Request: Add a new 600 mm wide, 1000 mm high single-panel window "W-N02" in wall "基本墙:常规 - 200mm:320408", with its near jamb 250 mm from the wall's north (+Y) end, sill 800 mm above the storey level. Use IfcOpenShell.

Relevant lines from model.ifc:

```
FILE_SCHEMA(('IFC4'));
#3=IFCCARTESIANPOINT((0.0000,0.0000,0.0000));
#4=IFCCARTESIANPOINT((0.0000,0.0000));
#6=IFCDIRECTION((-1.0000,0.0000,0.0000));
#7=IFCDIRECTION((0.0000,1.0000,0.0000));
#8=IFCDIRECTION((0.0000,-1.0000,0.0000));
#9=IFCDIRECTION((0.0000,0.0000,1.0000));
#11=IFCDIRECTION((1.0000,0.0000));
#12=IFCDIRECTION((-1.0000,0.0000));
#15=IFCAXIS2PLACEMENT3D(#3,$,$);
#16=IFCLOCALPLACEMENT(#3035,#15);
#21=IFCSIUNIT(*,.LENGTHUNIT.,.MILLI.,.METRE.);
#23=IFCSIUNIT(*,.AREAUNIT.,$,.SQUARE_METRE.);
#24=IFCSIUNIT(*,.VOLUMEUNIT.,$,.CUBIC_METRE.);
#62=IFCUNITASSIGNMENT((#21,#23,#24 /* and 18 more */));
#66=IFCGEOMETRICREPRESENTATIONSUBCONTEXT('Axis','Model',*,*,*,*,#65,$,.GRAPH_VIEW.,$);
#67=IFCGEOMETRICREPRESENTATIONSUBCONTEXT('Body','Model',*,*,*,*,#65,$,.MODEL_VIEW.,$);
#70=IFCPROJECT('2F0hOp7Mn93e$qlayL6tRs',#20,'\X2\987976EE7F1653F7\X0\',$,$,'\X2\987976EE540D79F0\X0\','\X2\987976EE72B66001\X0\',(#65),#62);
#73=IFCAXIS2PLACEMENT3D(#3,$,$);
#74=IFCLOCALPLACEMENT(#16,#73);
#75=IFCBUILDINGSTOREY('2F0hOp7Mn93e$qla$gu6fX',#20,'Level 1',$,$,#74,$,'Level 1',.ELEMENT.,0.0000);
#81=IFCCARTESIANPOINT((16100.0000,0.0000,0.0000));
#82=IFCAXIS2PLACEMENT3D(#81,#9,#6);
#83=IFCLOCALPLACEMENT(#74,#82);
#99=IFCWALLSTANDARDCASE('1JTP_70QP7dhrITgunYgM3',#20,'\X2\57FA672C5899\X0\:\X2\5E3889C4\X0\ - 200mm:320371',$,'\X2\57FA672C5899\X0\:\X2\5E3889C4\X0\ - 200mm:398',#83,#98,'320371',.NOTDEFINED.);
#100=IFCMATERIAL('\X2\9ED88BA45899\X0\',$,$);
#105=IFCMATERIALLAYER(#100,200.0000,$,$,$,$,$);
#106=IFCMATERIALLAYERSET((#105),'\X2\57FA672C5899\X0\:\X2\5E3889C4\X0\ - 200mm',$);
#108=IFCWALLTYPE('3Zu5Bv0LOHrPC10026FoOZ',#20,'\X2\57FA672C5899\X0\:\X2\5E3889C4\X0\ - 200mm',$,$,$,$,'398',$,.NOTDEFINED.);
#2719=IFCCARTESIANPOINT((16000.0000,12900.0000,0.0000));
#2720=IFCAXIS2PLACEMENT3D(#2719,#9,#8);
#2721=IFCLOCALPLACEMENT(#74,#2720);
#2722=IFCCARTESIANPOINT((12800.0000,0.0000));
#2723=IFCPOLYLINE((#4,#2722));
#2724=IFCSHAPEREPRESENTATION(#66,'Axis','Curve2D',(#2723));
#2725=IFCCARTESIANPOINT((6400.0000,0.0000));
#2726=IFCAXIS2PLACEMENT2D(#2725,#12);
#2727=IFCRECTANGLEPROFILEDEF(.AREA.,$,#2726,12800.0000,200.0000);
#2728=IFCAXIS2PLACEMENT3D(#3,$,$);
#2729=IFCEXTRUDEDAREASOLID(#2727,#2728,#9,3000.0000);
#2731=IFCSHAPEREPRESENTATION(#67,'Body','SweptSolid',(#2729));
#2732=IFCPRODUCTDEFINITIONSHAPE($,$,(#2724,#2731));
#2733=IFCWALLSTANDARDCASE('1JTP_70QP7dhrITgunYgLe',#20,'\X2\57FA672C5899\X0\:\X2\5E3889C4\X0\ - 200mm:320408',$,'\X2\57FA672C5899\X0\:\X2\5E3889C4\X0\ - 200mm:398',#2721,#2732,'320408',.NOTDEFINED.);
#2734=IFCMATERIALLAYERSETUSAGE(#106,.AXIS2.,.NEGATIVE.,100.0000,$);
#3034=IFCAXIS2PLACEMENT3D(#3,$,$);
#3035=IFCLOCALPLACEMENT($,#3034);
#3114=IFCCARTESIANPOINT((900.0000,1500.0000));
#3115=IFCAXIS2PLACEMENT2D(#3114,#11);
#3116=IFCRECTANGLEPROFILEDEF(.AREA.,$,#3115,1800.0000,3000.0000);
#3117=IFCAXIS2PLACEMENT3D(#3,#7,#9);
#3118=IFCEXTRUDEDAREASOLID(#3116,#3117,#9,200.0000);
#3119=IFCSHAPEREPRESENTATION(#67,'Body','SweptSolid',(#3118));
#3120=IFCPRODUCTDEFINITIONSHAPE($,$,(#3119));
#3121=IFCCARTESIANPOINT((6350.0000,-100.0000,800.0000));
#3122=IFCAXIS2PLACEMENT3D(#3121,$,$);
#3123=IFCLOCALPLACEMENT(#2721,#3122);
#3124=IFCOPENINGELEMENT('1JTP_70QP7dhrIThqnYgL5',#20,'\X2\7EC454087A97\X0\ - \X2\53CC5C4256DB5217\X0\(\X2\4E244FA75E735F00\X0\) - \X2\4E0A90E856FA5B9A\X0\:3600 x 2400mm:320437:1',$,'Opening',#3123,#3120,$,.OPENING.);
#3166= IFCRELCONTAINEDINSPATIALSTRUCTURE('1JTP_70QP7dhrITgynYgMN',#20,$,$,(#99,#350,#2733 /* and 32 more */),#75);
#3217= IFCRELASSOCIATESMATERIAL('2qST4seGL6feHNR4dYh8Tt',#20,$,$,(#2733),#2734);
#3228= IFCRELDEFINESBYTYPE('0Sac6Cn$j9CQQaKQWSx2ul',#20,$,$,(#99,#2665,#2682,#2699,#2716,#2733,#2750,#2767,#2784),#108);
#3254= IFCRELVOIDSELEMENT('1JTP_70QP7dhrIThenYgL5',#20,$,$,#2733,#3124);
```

```python
import numpy as np
import ifcopenshell
import ifcopenshell.api.feature
import ifcopenshell.api.geometry
import ifcopenshell.api.root
import ifcopenshell.api.spatial
import ifcopenshell.geom
import ifcopenshell.util.element
import ifcopenshell.util.placement
import ifcopenshell.util.representation
import ifcopenshell.util.shape
import ifcopenshell.util.unit

model = ifcopenshell.open("model.ifc")
unit_scale = ifcopenshell.util.unit.calculate_unit_scale(model)
settings = ifcopenshell.geom.settings()


def volume(element):
    """Net volume in cubic metres, openings subtracted."""
    shape = ifcopenshell.geom.create_shape(settings, element)
    return ifcopenshell.util.shape.get_volume(shape.geometry)


wall = model.by_guid("1JTP_70QP7dhrITgunYgLe")
storey = ifcopenshell.util.element.get_container(wall, ifc_class="IfcBuildingStorey")
context = ifcopenshell.util.representation.get_context(model, "Model", "Body", "MODEL_VIEW")
before = volume(wall)

width, height, from_end, sill = 0.6, 1, 0.25, 0.8  # metres

# The wall runs along its own X axis, and the end named is its -X end.
wall_shape = ifcopenshell.geom.create_shape(settings, wall)
x, y, z = ifcopenshell.util.shape.get_vertices(wall_shape.geometry).T
start = x.min() + from_end
face, thickness = float(y.min()), float(y.max() - y.min())
wall_matrix = ifcopenshell.util.placement.get_local_placement(wall.ObjectPlacement)
level = ifcopenshell.util.placement.get_local_placement(storey.ObjectPlacement)[2, 3]


def in_wall(x, y):
    """Placement at x, y metres in the wall's axes, at sill height."""
    matrix = wall_matrix.copy()
    matrix[:, 3] = wall_matrix @ np.array([x / unit_scale, y / unit_scale, 0.0, 1.0])
    matrix[2, 3] = level + sill / unit_scale
    return matrix


# Opening: a box that overshoots both wall faces by 50 mm.
opening = ifcopenshell.api.root.create_entity(model, ifc_class="IfcOpeningElement", predefined_type="OPENING")
box = ifcopenshell.api.geometry.add_wall_representation(
    model, context=context, length=width, height=height, thickness=thickness + 0.1
)
ifcopenshell.api.geometry.assign_representation(model, product=opening, representation=box)
ifcopenshell.api.geometry.edit_object_placement(model, product=opening, matrix=in_wall(start, face - 0.05), is_si=False)
ifcopenshell.api.feature.add_feature(model, feature=opening, element=wall)

window = ifcopenshell.api.root.create_entity(model, ifc_class="IfcWindow", name="W-N02", predefined_type="WINDOW")
window.OverallWidth, window.OverallHeight = width / unit_scale, height / unit_scale
window.PartitioningType = "SINGLE_PANEL"
body = ifcopenshell.api.geometry.add_window_representation(
    model,
    context=context,
    overall_width=window.OverallWidth,
    overall_height=window.OverallHeight,
    partition_type="SINGLE_PANEL",
)
ifcopenshell.api.geometry.assign_representation(model, product=window, representation=body)
ifcopenshell.api.spatial.assign_container(model, products=[window], relating_structure=storey)
ifcopenshell.api.feature.add_filling(model, opening=opening, element=window)

# Centre the window in the wall's thickness.
ifcopenshell.api.geometry.edit_object_placement(model, product=window, matrix=in_wall(start, face), is_si=False)
window_shape = ifcopenshell.geom.create_shape(settings, window)
depth = ifcopenshell.util.shape.get_vertices(window_shape.geometry)[:, 1]
offset = face + thickness / 2 - (depth.min() + depth.max()) / 2
ifcopenshell.api.geometry.edit_object_placement(model, product=window, matrix=in_wall(start, offset), is_si=False)

after = volume(wall)

print(f"wall volume {before:.3f} -> {after:.3f} m3")

model.write("model-out.ifc")
```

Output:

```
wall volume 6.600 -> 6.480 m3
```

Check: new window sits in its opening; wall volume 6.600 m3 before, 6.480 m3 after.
